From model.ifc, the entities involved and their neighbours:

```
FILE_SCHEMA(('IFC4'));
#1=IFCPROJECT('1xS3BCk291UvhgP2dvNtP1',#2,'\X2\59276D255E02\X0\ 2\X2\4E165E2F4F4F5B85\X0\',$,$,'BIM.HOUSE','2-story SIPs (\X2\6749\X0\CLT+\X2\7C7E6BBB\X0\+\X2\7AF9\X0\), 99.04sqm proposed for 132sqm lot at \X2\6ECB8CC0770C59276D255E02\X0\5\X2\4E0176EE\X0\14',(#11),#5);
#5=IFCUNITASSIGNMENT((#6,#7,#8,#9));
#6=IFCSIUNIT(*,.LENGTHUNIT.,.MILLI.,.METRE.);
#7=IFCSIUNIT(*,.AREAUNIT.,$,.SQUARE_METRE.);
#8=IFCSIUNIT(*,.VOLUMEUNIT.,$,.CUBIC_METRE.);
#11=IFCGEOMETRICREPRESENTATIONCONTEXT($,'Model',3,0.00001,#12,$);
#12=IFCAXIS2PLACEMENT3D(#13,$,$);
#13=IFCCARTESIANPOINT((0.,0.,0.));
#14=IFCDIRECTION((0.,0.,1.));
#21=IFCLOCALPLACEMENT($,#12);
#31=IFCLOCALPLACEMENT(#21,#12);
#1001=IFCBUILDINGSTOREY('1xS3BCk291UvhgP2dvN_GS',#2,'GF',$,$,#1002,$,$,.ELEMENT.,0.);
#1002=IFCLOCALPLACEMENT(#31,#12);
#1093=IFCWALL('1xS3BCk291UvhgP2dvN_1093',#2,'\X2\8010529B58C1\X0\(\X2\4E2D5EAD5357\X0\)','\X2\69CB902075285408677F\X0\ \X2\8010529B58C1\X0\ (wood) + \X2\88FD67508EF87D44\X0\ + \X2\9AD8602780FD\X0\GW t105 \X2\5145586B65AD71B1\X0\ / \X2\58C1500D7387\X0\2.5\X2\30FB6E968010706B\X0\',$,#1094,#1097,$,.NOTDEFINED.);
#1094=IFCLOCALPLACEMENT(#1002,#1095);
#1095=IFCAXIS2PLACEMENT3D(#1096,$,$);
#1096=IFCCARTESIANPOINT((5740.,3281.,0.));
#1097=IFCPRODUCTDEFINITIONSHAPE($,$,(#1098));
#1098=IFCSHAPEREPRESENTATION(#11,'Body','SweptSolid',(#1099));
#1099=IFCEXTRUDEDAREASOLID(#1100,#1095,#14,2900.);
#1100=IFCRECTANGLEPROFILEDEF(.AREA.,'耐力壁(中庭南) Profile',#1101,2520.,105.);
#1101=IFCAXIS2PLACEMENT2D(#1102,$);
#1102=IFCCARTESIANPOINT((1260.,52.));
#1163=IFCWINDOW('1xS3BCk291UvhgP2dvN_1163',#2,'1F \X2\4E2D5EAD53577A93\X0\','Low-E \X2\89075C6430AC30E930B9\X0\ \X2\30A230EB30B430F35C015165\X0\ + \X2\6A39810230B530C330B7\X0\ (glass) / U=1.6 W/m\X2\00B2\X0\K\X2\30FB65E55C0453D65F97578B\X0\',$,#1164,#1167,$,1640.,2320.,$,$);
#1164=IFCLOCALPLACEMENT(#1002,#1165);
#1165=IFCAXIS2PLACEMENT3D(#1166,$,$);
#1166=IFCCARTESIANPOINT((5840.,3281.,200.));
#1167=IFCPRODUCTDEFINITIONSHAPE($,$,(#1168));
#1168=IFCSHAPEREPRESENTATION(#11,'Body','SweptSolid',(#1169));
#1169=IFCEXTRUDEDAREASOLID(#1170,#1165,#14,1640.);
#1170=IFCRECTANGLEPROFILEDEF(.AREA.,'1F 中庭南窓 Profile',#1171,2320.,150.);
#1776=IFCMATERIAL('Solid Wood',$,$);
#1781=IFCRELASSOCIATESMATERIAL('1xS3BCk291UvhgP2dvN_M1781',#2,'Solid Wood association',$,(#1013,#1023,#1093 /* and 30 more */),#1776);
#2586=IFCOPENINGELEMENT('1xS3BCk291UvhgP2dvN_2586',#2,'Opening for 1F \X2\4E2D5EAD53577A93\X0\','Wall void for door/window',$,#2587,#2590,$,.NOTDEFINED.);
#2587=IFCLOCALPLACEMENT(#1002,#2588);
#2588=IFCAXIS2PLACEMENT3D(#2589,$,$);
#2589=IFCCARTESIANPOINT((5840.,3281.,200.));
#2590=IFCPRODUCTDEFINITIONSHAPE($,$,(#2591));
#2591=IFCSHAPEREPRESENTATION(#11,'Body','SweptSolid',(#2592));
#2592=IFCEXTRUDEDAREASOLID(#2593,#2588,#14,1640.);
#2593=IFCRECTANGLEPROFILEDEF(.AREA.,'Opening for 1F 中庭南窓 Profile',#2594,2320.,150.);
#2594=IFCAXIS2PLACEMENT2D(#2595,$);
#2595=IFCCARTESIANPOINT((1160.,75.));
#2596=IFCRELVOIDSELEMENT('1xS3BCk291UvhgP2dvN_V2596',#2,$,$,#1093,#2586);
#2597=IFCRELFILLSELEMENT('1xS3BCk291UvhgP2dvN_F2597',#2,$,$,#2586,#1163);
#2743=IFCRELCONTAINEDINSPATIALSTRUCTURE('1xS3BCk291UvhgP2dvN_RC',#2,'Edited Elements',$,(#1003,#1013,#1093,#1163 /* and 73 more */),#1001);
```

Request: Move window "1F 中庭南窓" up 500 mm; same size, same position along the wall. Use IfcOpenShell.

```python
import numpy as np
import ifcopenshell
import ifcopenshell.api.geometry
import ifcopenshell.util.placement
import ifcopenshell.util.unit

model = ifcopenshell.open("model.ifc")
unit_scale = ifcopenshell.util.unit.calculate_unit_scale(model)

window = model.by_guid("1xS3BCk291UvhgP2dvN_1163")
opening = window.FillsVoids[0].RelatingOpeningElement
dz = 0.5 / unit_scale

shift = np.array([0.0, 0.0, dz])
# The window is not placed relative to its opening, so move both.
for product in (opening, window):
    matrix = ifcopenshell.util.placement.get_local_placement(product.ObjectPlacement)
    matrix[:3, 3] += shift
    ifcopenshell.api.geometry.edit_object_placement(model, product=product, matrix=matrix, is_si=False)

print(f"moved by {dz * unit_scale:+.3f} m")

model.write("model_v2.ifc")
```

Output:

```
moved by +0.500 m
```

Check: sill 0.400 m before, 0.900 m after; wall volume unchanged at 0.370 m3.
